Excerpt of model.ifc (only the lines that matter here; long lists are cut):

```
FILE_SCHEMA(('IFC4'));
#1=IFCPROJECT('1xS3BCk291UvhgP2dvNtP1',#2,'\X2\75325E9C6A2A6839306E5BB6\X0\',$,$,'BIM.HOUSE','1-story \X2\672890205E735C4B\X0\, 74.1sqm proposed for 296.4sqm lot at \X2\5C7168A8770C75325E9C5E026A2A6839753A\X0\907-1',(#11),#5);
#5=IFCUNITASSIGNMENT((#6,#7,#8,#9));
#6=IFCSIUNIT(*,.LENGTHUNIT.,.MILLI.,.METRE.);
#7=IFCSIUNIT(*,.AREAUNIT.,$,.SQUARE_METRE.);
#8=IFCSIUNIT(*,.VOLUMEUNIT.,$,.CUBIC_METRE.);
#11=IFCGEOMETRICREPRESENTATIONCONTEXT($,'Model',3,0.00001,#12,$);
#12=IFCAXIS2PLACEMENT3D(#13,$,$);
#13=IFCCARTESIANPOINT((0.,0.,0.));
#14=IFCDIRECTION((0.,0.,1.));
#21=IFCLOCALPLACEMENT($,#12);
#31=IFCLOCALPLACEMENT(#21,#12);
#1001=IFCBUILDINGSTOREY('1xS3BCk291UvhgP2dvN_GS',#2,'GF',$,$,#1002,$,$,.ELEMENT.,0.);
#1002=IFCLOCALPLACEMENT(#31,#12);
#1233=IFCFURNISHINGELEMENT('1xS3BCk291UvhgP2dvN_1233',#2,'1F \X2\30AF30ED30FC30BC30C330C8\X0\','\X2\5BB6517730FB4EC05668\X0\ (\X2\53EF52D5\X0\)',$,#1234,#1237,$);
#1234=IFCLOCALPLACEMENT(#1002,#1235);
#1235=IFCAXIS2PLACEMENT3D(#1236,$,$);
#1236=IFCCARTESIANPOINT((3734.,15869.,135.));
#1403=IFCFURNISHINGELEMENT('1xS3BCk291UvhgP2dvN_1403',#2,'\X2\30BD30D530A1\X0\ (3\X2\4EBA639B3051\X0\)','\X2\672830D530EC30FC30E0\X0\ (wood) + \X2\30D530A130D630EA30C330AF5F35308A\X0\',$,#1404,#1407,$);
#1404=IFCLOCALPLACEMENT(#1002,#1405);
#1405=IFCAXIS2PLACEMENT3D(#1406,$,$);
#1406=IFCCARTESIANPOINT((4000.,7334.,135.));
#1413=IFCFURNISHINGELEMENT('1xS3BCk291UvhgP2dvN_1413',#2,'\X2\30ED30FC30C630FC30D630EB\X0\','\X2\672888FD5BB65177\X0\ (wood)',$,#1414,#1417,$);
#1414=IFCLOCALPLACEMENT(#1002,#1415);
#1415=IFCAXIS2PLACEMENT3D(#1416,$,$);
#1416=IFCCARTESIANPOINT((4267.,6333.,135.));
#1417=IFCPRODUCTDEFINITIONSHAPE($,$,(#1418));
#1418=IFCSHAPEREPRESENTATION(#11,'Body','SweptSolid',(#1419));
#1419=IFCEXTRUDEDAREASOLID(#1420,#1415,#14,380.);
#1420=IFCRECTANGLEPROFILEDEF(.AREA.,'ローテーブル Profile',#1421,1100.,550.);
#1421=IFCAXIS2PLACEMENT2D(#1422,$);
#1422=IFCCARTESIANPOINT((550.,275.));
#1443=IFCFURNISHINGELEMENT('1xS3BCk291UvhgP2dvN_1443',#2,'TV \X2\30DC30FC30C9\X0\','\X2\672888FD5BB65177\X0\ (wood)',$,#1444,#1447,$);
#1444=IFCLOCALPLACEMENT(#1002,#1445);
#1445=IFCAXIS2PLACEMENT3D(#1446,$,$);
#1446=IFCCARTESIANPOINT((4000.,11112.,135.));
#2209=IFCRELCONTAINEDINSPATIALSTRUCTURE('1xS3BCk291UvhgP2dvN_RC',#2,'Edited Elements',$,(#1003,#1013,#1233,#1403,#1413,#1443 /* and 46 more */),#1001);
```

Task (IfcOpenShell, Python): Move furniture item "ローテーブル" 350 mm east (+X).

```python
import ifcopenshell
import ifcopenshell.api.geometry
import ifcopenshell.util.placement
import ifcopenshell.util.unit

model = ifcopenshell.open("model.ifc")
unit_scale = ifcopenshell.util.unit.calculate_unit_scale(model)

item = model.by_guid("1xS3BCk291UvhgP2dvN_1413")
matrix = ifcopenshell.util.placement.get_local_placement(item.ObjectPlacement)
matrix[0, 3] += 0.35 / unit_scale
ifcopenshell.api.geometry.edit_object_placement(model, product=item, matrix=matrix, is_si=False)

print(ifcopenshell.util.placement.get_local_placement(item.ObjectPlacement).round(3) + 0.0)

model.write("model_edited.ifc")
```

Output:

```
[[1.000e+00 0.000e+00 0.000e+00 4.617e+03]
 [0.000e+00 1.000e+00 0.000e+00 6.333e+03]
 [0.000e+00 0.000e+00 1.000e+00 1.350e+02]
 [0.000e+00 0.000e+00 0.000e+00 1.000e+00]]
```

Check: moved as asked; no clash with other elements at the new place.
